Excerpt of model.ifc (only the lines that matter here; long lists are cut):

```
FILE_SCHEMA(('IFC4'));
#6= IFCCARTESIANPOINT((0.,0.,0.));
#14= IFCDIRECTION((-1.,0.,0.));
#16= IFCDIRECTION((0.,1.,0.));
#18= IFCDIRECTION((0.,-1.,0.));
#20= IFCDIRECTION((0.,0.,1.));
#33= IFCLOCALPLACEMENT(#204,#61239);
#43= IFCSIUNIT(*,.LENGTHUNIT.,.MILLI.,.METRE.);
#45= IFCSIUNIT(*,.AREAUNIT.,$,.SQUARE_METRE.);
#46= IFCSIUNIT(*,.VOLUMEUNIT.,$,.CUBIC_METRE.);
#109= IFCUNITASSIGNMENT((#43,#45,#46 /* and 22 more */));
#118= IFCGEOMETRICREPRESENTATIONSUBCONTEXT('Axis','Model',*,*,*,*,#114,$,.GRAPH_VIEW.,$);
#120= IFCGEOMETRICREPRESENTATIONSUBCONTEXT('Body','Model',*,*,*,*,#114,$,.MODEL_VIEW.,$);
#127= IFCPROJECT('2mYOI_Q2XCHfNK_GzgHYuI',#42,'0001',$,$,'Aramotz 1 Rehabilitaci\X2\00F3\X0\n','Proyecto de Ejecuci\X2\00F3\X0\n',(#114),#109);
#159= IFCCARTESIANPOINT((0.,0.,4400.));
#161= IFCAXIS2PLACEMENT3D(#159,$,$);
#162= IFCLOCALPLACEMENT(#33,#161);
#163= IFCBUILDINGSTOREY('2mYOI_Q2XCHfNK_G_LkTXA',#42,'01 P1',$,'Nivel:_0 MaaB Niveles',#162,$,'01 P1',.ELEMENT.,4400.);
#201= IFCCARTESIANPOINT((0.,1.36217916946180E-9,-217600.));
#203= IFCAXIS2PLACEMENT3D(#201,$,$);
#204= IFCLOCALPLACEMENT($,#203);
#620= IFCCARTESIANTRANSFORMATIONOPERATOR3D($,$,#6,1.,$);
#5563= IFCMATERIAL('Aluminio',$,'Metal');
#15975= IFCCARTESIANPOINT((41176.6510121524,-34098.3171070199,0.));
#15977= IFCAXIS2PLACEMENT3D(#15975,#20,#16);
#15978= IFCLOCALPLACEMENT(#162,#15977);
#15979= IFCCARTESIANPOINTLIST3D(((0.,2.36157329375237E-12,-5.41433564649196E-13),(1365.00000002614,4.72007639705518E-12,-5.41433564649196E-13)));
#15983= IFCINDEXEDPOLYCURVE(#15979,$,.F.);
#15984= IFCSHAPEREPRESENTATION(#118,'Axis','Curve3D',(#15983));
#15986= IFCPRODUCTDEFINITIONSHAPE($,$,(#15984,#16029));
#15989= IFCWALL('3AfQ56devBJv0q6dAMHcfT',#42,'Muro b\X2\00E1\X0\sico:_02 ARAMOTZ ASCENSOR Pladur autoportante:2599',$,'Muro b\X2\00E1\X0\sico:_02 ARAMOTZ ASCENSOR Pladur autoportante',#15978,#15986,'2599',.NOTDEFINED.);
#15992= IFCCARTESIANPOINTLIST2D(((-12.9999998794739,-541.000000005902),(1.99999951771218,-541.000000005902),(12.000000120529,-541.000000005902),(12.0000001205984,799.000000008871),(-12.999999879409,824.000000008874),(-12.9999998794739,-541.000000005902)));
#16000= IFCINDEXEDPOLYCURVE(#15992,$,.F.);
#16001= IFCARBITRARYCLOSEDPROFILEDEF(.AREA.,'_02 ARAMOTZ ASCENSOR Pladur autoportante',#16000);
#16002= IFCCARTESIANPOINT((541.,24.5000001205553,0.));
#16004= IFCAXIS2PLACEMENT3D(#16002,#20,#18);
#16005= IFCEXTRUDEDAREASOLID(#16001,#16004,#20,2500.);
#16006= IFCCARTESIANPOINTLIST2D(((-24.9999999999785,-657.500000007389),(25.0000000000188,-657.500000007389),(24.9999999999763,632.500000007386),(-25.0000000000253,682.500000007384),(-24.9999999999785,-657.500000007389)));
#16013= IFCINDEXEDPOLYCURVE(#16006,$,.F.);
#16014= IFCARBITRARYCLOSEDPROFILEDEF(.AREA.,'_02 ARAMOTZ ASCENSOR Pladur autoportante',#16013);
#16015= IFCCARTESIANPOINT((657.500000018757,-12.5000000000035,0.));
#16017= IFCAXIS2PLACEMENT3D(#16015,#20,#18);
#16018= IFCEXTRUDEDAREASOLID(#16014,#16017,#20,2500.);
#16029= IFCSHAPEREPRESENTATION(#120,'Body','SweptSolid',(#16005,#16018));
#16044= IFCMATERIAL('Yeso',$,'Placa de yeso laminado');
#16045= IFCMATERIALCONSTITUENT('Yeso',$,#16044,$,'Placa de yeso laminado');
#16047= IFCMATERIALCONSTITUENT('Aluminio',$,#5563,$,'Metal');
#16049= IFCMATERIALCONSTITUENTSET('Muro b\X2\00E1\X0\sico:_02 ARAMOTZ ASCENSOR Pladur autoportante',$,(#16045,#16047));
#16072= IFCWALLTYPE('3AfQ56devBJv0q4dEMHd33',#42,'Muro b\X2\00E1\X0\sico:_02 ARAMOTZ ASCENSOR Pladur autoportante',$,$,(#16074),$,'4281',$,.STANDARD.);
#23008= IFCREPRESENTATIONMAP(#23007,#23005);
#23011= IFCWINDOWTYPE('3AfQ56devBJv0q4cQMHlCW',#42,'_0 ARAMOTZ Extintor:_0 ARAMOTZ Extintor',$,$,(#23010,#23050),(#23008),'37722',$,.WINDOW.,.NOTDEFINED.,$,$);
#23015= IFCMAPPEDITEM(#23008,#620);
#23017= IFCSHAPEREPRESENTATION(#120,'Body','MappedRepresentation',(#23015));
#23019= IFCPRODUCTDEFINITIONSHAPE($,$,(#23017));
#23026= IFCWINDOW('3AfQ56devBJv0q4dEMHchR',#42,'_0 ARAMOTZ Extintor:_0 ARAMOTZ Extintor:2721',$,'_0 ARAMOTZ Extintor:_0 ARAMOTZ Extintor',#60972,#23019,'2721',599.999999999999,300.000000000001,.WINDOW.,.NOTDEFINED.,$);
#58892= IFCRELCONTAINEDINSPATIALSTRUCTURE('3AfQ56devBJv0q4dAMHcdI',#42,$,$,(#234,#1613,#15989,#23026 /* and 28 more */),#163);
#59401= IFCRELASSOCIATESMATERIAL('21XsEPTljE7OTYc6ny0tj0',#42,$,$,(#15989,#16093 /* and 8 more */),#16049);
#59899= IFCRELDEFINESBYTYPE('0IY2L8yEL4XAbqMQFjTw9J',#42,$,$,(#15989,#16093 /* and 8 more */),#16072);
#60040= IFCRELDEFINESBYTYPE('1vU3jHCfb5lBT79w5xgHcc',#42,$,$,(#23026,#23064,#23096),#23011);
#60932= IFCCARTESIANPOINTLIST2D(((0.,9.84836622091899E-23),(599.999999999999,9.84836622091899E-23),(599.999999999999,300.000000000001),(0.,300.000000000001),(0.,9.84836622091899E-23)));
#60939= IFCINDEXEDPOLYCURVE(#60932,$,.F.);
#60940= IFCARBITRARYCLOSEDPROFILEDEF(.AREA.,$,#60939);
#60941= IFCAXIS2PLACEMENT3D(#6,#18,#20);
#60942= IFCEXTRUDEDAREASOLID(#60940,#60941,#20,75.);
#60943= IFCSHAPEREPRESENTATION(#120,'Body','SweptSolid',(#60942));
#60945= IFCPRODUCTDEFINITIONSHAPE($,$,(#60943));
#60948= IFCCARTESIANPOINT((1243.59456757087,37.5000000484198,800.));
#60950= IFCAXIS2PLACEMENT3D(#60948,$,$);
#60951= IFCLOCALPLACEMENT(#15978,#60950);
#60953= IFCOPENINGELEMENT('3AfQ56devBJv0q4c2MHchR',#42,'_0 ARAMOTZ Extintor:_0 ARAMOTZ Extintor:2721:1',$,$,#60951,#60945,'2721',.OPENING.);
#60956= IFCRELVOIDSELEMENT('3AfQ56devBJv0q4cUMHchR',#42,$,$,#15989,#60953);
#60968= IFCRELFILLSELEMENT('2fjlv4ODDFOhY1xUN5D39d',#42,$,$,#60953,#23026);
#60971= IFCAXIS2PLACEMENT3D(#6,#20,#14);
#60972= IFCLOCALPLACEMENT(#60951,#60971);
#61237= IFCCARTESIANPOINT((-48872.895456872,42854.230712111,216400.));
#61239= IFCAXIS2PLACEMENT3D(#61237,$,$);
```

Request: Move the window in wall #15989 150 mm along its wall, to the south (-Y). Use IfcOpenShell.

```python
import ifcopenshell
import ifcopenshell.api.geometry
import ifcopenshell.util.placement
import ifcopenshell.util.unit

model = ifcopenshell.open("model.ifc")
unit_scale = ifcopenshell.util.unit.calculate_unit_scale(model)

window = model.by_guid("3AfQ56devBJv0q4dEMHchR")
opening = window.FillsVoids[0].RelatingOpeningElement
wall = opening.VoidsElements[0].RelatingBuildingElement

wall_matrix = ifcopenshell.util.placement.get_local_placement(wall.ObjectPlacement)
shift = wall_matrix[:3, 0] * -0.15 / unit_scale
before = ifcopenshell.util.placement.get_local_placement(window.ObjectPlacement)[:3, 3].copy()

# The window is placed relative to its opening, so it follows when the opening moves.
matrix = ifcopenshell.util.placement.get_local_placement(opening.ObjectPlacement)
matrix[:3, 3] += shift
ifcopenshell.api.geometry.edit_object_placement(
    model, product=opening, matrix=matrix, is_si=False, should_transform_children=True
)

after = ifcopenshell.util.placement.get_local_placement(window.ObjectPlacement)[:3, 3]
print("window moved by", (after - before).round(3) + 0.0)

model.write("model-out.ifc")
```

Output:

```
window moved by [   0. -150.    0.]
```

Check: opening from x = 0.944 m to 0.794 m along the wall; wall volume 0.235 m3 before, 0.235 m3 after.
